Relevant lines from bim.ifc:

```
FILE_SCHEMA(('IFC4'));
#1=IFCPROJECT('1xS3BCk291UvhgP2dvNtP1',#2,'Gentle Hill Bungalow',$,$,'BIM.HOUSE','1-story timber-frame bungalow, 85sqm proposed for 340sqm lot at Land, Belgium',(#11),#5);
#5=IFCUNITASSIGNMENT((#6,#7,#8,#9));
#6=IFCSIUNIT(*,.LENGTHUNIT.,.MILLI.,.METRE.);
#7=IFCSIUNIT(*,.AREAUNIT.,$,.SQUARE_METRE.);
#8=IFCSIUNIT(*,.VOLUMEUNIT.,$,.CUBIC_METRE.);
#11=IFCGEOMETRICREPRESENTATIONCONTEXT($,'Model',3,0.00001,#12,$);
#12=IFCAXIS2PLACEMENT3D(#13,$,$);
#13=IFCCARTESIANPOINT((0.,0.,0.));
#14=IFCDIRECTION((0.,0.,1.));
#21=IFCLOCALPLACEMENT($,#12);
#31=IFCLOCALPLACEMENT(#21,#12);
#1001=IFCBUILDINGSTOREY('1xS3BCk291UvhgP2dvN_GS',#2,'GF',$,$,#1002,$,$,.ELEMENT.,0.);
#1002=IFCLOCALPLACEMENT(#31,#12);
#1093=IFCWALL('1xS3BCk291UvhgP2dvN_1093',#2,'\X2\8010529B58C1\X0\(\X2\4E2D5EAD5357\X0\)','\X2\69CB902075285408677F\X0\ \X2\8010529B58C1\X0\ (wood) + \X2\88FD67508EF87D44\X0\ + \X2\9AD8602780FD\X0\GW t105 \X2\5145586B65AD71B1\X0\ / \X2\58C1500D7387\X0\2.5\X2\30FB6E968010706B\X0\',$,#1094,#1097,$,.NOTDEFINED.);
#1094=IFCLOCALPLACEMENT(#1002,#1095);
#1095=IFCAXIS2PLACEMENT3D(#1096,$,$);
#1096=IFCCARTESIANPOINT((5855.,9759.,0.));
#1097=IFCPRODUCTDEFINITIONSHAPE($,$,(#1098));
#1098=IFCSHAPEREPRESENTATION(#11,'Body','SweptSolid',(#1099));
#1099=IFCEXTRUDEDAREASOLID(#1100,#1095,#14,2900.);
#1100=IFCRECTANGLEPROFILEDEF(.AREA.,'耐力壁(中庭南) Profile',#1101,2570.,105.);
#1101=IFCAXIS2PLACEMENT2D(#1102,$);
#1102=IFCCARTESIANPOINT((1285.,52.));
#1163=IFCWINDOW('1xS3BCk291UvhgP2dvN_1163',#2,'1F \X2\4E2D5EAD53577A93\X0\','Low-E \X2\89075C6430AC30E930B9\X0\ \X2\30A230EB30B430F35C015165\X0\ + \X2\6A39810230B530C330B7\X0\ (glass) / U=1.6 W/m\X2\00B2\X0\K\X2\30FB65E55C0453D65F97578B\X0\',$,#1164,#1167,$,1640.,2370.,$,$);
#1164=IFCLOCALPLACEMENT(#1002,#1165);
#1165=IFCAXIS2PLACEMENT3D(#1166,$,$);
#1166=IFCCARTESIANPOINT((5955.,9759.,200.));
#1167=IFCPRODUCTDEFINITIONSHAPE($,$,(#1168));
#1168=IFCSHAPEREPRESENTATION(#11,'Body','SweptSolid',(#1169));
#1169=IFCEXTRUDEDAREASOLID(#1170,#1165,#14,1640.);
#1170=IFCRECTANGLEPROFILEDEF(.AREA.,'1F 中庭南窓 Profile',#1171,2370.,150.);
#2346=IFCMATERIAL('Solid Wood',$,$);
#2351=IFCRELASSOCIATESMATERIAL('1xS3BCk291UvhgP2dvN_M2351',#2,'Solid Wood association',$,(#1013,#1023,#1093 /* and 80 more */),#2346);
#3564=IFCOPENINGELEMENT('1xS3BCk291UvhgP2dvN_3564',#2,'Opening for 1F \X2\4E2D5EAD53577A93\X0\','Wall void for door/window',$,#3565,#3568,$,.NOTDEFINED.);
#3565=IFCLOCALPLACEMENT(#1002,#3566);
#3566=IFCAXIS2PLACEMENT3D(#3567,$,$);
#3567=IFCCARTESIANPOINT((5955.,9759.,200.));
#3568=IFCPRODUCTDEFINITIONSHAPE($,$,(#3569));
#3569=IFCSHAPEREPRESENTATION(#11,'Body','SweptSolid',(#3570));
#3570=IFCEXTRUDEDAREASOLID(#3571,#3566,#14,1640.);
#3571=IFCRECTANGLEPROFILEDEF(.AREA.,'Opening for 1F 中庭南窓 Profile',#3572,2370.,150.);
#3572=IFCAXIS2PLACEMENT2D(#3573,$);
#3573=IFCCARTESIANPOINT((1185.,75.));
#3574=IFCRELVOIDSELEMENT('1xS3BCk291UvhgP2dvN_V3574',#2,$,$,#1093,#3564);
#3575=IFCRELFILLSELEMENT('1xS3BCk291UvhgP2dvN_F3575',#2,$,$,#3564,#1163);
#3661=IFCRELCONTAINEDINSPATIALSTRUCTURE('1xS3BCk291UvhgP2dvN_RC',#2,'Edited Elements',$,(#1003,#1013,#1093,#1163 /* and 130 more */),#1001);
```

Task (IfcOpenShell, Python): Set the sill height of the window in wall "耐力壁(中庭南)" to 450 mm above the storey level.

```python
import numpy as np
import ifcopenshell
import ifcopenshell.api.geometry
import ifcopenshell.geom
import ifcopenshell.util.element
import ifcopenshell.util.placement
import ifcopenshell.util.shape
import ifcopenshell.util.unit

model = ifcopenshell.open("bim.ifc")
unit_scale = ifcopenshell.util.unit.calculate_unit_scale(model)

window = model.by_guid("1xS3BCk291UvhgP2dvN_1163")
opening = window.FillsVoids[0].RelatingOpeningElement
storey = ifcopenshell.util.element.get_container(window, ifc_class="IfcBuildingStorey")
level = ifcopenshell.util.placement.get_local_placement(storey.ObjectPlacement)[2, 3]

# The opening's origin need not be at the sill, so measure its lowest point.
shape = ifcopenshell.geom.create_shape(ifcopenshell.geom.settings(), opening)
bottom = ifcopenshell.util.shape.get_shape_bottom_elevation(shape, shape.geometry) / unit_scale
dz = level + 0.45 / unit_scale - bottom

shift = np.array([0.0, 0.0, dz])
# The window is not placed relative to its opening, so move both.
for product in (opening, window):
    matrix = ifcopenshell.util.placement.get_local_placement(product.ObjectPlacement)
    matrix[:3, 3] += shift
    ifcopenshell.api.geometry.edit_object_placement(model, product=product, matrix=matrix, is_si=False)

print(f"moved by {dz * unit_scale:+.3f} m")

model.write("bim_v2.ifc")
```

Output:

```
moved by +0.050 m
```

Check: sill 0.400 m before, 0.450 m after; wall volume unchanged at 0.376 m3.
